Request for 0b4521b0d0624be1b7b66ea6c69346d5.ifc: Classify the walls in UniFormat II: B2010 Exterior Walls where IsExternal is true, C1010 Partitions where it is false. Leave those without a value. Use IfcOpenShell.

First a look at what the model holds.

```python
import ifcopenshell
import ifcopenshell.util.element

model = ifcopenshell.open("0b4521b0d0624be1b7b66ea6c69346d5.ifc")
print(model.schema)
print("classifications:", [c.Name for c in model.by_type("IfcClassification")])
values = [ifcopenshell.util.element.get_pset(e, "Pset_WallCommon", "IsExternal") for e in model.by_type("IfcWall")]
for value in (True, False, None):
    print("IsExternal", value, values.count(value))
```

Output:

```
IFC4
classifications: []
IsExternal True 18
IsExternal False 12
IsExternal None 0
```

```python
import ifcopenshell
import ifcopenshell.api.classification
import ifcopenshell.util.element

model = ifcopenshell.open("0b4521b0d0624be1b7b66ea6c69346d5.ifc")

system = ifcopenshell.api.classification.add_classification(model, classification="UniFormat II")

walls = model.by_type("IfcWall")
external = {e: ifcopenshell.util.element.get_pset(e, "Pset_WallCommon", "IsExternal") for e in walls}
for flag, code, name in ((True, "B2010", "Exterior Walls"), (False, "C1010", "Partitions")):
    products = [e for e in walls if external[e] is flag]
    ifcopenshell.api.classification.add_reference(
        model, products=products, classification=system, identification=code, name=name
    )
    print(code, len(products))

model.write("0b4521b0d0624be1b7b66ea6c69346d5_v2.ifc")
```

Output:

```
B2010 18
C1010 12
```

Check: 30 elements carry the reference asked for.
